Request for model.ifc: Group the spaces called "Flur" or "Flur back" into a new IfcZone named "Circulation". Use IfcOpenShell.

First a look at what the model holds.

```python
import ifcopenshell

model = ifcopenshell.open("model.ifc")
print(model.schema)
seen = {}
for space in model.by_type("IfcSpace"):
    seen[space.LongName] = seen.get(space.LongName, 0) + 1
for name, count in sorted(seen.items(), key=str):
    print(count, "x", name)
print("zones:", [z.Name for z in model.by_type("IfcZone")][:20])
```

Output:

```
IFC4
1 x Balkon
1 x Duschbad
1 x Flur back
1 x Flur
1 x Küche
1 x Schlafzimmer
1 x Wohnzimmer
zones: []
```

```python
import ifcopenshell
import ifcopenshell.api.group
import ifcopenshell.api.root

model = ifcopenshell.open("model.ifc")

names = {"Flur", "Flur back"}
spaces = [s for s in model.by_type("IfcSpace") if s.LongName in names]

zone = ifcopenshell.api.root.create_entity(model, ifc_class="IfcZone", name="Circulation")
ifcopenshell.api.group.assign_group(model, products=spaces, group=zone)
print(len(spaces), "spaces in", zone.Name)

model.write("model_rev.ifc")
```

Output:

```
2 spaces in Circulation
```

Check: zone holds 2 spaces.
